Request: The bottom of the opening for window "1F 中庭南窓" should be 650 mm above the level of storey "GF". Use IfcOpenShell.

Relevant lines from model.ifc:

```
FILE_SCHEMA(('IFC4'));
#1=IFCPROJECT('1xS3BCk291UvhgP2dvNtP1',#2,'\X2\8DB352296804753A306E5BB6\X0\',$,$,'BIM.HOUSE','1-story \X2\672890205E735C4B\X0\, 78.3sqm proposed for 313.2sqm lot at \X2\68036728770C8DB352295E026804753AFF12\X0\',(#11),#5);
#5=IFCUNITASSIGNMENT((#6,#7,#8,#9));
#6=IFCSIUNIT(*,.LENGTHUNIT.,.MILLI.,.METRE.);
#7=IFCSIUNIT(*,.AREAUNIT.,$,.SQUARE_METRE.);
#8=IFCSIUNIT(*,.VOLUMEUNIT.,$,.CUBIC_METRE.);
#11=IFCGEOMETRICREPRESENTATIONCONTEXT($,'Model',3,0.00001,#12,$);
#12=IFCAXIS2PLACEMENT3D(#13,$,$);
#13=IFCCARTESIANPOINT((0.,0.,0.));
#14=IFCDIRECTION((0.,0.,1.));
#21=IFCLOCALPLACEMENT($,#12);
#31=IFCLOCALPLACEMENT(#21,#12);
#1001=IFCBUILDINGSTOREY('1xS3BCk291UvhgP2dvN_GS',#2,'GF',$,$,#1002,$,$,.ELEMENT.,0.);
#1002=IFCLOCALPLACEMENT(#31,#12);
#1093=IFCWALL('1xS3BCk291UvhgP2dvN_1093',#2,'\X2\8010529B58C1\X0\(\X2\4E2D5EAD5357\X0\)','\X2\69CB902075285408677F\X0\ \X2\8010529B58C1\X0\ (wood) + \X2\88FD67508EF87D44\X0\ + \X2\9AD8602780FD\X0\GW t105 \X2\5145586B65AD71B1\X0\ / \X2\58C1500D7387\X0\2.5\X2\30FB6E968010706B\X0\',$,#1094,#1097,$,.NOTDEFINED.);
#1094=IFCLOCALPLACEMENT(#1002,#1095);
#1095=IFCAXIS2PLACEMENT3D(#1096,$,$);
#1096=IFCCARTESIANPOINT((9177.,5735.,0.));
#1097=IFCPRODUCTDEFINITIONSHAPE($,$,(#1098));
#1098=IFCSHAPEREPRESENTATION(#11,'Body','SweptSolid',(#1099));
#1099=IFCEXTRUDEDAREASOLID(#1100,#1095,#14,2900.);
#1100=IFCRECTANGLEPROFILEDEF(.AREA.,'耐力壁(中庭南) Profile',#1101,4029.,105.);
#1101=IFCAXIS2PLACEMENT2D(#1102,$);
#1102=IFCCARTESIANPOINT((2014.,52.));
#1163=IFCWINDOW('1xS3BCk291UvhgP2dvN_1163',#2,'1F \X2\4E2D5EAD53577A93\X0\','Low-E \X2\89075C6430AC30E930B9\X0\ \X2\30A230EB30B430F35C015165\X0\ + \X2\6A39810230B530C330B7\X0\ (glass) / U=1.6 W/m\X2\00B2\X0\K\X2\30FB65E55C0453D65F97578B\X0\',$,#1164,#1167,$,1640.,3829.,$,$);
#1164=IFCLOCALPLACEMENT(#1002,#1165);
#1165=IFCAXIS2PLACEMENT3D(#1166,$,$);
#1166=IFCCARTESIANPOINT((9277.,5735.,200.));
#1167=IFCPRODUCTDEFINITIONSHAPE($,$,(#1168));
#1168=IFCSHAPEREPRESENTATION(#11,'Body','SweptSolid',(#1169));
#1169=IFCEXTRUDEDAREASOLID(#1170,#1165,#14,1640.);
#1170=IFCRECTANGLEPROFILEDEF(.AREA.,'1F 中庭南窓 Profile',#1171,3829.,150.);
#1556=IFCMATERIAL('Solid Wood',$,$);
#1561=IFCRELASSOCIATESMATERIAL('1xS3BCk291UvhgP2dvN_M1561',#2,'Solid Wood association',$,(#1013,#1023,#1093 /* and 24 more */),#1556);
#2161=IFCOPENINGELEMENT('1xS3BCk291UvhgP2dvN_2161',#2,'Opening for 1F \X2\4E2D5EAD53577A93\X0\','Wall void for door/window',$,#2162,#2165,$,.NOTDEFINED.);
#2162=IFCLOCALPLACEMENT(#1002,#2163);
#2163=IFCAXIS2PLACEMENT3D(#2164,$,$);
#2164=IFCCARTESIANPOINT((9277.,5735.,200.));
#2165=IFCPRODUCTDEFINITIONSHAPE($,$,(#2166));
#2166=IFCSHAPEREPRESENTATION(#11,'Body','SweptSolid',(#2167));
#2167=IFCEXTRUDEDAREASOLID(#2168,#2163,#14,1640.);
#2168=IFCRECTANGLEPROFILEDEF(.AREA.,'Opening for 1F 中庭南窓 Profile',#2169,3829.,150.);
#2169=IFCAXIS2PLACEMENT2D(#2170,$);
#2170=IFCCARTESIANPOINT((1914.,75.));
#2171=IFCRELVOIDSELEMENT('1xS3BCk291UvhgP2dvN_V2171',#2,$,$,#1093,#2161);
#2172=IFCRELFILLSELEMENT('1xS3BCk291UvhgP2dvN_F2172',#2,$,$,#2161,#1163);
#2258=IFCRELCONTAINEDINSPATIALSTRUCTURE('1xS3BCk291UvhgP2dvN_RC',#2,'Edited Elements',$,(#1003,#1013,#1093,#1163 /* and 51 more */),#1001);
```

```python
import numpy as np
import ifcopenshell
import ifcopenshell.api.geometry
import ifcopenshell.geom
import ifcopenshell.util.element
import ifcopenshell.util.placement
import ifcopenshell.util.shape
import ifcopenshell.util.unit

model = ifcopenshell.open("model.ifc")
unit_scale = ifcopenshell.util.unit.calculate_unit_scale(model)

window = model.by_guid("1xS3BCk291UvhgP2dvN_1163")
opening = window.FillsVoids[0].RelatingOpeningElement
storey = ifcopenshell.util.element.get_container(window, ifc_class="IfcBuildingStorey")
level = ifcopenshell.util.placement.get_local_placement(storey.ObjectPlacement)[2, 3]

# The opening's origin need not be at the sill, so measure its lowest point.
shape = ifcopenshell.geom.create_shape(ifcopenshell.geom.settings(), opening)
bottom = ifcopenshell.util.shape.get_shape_bottom_elevation(shape, shape.geometry) / unit_scale
dz = level + 650.0 - bottom

shift = np.array([0.0, 0.0, dz])
# The window is not placed relative to its opening, so move both.
for product in (opening, window):
    matrix = ifcopenshell.util.placement.get_local_placement(product.ObjectPlacement)
    matrix[:3, 3] += shift
    ifcopenshell.api.geometry.edit_object_placement(model, product=product, matrix=matrix, is_si=False)

print(f"moved by {dz * unit_scale:+.3f} m")

model.write("model_edited.ifc")
```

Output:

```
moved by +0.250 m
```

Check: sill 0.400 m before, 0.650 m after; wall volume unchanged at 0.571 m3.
